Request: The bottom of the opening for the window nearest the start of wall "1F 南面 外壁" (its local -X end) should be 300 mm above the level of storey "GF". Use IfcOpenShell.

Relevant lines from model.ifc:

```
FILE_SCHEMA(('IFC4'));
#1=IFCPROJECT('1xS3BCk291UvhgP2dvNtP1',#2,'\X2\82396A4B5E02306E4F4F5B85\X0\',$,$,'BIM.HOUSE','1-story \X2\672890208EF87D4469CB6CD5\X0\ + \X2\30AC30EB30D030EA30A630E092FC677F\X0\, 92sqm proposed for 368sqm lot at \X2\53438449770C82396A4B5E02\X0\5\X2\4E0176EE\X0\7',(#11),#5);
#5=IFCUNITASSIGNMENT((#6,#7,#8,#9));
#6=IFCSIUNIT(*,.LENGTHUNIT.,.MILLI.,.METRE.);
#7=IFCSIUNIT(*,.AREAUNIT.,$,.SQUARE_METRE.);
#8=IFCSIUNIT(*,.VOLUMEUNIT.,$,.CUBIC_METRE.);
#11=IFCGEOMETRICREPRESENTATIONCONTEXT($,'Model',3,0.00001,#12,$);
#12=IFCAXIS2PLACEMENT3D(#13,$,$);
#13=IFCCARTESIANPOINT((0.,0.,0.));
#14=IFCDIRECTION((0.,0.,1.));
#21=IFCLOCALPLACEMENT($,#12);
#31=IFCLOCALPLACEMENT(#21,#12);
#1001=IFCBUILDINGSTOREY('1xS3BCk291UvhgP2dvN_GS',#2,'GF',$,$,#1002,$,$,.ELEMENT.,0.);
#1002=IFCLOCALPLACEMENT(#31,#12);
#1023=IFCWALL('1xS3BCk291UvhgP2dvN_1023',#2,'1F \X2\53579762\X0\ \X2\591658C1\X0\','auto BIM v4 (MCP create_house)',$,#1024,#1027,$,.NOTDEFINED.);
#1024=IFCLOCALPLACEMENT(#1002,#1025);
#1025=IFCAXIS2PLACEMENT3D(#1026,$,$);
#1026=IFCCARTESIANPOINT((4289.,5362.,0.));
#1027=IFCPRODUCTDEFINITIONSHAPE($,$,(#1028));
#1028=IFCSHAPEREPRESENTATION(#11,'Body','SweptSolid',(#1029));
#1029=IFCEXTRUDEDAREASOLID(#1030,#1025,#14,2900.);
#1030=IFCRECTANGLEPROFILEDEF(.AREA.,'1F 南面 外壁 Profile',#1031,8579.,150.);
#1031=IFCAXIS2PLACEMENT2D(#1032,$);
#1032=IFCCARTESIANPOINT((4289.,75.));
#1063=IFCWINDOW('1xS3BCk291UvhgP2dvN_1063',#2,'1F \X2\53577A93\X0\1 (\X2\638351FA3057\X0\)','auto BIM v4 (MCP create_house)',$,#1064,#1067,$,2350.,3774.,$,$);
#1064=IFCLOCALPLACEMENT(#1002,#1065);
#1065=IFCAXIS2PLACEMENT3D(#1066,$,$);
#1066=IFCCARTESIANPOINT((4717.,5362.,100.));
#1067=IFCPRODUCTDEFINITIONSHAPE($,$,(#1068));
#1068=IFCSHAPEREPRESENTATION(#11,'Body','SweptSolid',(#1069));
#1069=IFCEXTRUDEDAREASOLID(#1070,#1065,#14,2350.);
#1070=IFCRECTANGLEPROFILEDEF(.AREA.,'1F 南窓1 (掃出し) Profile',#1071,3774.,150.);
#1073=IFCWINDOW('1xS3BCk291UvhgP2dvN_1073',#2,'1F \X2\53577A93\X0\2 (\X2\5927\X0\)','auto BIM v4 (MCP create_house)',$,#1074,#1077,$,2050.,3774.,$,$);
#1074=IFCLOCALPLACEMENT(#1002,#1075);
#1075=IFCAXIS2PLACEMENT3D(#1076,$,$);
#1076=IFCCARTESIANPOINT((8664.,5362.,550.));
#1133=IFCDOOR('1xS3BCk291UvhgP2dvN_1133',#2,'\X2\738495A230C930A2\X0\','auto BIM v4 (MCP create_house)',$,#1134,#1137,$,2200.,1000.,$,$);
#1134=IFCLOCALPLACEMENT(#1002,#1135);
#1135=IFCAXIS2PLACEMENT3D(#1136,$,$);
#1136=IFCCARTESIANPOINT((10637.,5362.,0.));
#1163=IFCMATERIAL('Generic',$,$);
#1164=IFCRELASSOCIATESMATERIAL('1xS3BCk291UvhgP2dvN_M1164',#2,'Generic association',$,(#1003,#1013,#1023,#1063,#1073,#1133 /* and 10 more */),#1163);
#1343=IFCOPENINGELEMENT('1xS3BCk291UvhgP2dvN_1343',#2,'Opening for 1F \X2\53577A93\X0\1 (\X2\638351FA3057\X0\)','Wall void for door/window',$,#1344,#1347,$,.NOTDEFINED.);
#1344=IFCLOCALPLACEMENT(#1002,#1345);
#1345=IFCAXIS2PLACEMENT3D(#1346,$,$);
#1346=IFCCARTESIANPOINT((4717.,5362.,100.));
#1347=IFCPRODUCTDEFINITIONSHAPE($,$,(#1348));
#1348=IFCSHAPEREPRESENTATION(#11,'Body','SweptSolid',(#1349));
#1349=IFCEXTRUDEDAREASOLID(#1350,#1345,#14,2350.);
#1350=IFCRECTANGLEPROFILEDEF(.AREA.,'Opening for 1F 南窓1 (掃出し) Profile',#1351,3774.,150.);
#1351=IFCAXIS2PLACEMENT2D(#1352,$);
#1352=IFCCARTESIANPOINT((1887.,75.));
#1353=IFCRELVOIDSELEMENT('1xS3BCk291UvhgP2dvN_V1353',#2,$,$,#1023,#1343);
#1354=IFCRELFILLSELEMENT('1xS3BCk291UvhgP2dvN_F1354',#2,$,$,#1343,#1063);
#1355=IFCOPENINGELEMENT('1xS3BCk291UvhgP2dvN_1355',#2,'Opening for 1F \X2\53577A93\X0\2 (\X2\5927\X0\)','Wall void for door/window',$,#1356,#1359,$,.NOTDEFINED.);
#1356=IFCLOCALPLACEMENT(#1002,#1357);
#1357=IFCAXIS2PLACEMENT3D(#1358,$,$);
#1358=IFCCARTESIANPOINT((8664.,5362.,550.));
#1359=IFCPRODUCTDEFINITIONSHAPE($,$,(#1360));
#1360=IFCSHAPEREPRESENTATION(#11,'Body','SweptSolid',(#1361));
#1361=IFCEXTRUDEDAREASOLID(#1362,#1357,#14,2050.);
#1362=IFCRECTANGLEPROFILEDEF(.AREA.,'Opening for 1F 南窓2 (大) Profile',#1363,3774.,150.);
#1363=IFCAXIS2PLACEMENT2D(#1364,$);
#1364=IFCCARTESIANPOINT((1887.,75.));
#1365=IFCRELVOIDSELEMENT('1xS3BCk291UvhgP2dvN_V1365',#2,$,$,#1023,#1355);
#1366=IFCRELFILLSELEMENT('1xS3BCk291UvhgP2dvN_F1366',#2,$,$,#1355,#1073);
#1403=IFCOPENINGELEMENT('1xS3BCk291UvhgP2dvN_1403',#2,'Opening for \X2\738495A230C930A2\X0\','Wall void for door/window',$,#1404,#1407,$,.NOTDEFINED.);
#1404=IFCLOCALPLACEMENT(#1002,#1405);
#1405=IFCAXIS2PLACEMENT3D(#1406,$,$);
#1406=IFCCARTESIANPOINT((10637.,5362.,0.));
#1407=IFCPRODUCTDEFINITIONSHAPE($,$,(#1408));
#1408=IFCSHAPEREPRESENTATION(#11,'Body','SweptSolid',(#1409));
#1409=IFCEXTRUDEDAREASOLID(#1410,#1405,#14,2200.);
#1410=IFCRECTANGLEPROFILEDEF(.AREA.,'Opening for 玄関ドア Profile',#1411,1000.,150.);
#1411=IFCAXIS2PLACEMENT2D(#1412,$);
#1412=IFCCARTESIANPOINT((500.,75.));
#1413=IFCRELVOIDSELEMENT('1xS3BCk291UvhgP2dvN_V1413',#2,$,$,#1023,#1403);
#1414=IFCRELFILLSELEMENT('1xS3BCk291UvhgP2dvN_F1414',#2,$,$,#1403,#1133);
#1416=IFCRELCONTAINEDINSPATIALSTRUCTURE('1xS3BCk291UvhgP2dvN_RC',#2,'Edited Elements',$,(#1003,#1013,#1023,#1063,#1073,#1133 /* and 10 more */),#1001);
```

```python
import numpy as np
import ifcopenshell
import ifcopenshell.api.geometry
import ifcopenshell.geom
import ifcopenshell.util.element
import ifcopenshell.util.placement
import ifcopenshell.util.shape
import ifcopenshell.util.unit

model = ifcopenshell.open("model.ifc")
unit_scale = ifcopenshell.util.unit.calculate_unit_scale(model)

window = model.by_guid("1xS3BCk291UvhgP2dvN_1063")
opening = window.FillsVoids[0].RelatingOpeningElement
storey = ifcopenshell.util.element.get_container(window, ifc_class="IfcBuildingStorey")
level = ifcopenshell.util.placement.get_local_placement(storey.ObjectPlacement)[2, 3]

# The opening's origin need not be at the sill, so measure its lowest point.
shape = ifcopenshell.geom.create_shape(ifcopenshell.geom.settings(), opening)
bottom = ifcopenshell.util.shape.get_shape_bottom_elevation(shape, shape.geometry) / unit_scale
dz = level + 0.3 / unit_scale - bottom

shift = np.array([0.0, 0.0, dz])
# The window is not placed relative to its opening, so move both.
for product in (opening, window):
    matrix = ifcopenshell.util.placement.get_local_placement(product.ObjectPlacement)
    matrix[:3, 3] += shift
    ifcopenshell.api.geometry.edit_object_placement(model, product=product, matrix=matrix, is_si=False)

print(f"moved by {dz * unit_scale:+.3f} m")

model.write("model_edited.ifc")
```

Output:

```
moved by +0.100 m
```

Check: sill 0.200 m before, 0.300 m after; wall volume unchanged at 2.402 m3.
